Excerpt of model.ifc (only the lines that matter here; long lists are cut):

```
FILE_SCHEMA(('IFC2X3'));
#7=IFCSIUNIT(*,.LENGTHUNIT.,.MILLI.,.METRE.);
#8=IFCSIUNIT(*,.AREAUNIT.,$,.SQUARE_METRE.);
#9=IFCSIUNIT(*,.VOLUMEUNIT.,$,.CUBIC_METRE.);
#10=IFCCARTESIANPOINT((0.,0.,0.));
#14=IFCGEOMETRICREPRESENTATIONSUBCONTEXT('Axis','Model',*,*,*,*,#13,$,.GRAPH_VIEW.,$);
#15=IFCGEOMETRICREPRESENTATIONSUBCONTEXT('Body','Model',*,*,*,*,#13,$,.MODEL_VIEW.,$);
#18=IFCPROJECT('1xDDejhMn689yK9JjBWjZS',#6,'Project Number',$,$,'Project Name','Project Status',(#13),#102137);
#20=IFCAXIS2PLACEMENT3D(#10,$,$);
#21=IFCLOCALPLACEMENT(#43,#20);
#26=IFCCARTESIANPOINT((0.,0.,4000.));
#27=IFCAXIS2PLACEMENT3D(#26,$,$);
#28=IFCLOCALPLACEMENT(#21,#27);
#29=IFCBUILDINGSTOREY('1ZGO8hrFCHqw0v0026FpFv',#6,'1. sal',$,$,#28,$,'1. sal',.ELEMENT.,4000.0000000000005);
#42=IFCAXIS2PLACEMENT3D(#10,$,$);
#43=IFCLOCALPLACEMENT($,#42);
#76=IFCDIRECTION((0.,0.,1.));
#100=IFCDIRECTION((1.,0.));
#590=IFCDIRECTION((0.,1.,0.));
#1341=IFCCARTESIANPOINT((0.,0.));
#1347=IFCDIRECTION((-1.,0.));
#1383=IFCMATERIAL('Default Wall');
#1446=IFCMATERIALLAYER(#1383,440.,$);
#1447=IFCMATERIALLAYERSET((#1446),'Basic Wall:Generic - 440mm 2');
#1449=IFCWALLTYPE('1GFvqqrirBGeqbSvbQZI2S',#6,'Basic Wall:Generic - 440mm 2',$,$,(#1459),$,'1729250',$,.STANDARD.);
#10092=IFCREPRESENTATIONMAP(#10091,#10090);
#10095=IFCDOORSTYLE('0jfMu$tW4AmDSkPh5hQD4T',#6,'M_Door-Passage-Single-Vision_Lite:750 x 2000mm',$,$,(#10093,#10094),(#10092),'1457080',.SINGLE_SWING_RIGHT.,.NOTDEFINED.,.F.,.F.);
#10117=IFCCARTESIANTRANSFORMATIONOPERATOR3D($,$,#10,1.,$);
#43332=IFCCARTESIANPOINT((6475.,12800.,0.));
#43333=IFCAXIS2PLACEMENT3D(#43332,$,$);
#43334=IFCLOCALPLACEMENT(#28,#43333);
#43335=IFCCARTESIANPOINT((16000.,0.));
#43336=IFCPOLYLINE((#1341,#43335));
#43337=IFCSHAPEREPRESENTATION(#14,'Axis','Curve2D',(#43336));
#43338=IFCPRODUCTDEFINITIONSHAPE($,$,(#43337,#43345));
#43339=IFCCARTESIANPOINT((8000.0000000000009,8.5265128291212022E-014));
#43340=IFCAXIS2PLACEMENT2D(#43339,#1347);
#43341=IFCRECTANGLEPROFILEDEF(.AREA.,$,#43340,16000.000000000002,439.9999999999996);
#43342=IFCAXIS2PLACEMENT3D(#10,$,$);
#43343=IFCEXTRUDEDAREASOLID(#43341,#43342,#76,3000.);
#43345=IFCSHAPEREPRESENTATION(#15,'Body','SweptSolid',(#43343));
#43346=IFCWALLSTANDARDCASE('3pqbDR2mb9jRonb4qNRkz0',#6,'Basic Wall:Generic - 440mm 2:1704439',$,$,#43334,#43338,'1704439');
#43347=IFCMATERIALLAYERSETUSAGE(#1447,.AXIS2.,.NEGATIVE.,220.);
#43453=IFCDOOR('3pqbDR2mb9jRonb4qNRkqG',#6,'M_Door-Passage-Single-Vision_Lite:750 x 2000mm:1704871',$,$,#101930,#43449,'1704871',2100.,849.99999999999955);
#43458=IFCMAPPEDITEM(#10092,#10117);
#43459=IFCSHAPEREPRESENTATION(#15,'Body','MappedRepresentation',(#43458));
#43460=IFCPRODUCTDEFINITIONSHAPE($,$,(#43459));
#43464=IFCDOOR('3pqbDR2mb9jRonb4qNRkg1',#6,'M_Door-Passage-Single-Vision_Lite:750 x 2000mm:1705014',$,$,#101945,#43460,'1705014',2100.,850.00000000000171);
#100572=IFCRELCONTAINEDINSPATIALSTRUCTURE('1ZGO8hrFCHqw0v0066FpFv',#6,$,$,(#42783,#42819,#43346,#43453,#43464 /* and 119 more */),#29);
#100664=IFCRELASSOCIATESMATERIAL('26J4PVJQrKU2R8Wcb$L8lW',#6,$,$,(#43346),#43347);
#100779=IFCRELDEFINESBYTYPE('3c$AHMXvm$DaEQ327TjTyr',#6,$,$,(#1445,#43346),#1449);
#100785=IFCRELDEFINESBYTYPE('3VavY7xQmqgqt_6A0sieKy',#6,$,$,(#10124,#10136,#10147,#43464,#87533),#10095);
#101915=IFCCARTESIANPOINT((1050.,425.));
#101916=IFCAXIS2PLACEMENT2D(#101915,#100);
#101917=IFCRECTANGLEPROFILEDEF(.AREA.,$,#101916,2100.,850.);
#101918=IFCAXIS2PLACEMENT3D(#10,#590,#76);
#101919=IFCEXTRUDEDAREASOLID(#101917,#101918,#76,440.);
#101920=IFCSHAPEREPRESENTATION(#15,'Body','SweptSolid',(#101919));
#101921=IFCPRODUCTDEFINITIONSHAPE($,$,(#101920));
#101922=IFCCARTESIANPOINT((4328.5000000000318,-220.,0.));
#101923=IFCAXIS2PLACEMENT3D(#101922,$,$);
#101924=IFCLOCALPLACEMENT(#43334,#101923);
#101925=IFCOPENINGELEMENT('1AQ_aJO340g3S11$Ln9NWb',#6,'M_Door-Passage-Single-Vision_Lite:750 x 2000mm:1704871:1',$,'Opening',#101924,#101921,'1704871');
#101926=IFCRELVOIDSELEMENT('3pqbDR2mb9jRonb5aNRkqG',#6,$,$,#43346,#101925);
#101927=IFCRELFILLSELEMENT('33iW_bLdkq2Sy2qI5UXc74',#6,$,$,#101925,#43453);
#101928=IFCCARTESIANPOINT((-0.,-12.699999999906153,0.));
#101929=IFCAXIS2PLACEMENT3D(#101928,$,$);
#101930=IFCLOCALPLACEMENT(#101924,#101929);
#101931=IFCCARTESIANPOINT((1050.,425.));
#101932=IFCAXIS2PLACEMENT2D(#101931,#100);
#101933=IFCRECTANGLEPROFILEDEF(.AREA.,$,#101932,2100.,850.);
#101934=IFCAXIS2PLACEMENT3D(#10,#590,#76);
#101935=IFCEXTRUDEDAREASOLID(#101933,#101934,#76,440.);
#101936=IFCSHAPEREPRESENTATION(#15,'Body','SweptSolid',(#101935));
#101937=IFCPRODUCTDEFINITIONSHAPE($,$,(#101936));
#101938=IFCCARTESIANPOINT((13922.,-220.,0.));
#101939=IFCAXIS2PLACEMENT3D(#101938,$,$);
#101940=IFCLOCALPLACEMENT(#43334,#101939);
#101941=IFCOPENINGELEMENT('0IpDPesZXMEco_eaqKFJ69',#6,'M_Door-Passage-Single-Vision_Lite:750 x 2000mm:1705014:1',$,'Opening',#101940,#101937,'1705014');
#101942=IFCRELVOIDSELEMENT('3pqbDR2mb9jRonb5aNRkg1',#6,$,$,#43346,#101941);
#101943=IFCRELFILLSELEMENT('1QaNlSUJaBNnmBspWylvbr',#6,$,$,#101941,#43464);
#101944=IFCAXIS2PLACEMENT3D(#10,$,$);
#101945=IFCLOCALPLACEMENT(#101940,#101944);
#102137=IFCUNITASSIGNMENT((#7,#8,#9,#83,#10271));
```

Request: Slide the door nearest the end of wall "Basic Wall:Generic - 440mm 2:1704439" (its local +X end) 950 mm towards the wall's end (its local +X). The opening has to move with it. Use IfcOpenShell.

```python
import ifcopenshell
import ifcopenshell.api.geometry
import ifcopenshell.util.placement
import ifcopenshell.util.unit

model = ifcopenshell.open("model.ifc")
unit_scale = ifcopenshell.util.unit.calculate_unit_scale(model)

door = model.by_guid("3pqbDR2mb9jRonb4qNRkg1")
opening = door.FillsVoids[0].RelatingOpeningElement
wall = opening.VoidsElements[0].RelatingBuildingElement

wall_matrix = ifcopenshell.util.placement.get_local_placement(wall.ObjectPlacement)
shift = wall_matrix[:3, 0] * 0.95 / unit_scale
before = ifcopenshell.util.placement.get_local_placement(door.ObjectPlacement)[:3, 3].copy()

# The door is placed relative to its opening, so it follows when the opening moves.
matrix = ifcopenshell.util.placement.get_local_placement(opening.ObjectPlacement)
matrix[:3, 3] += shift
ifcopenshell.api.geometry.edit_object_placement(
    model, product=opening, matrix=matrix, is_si=False, should_transform_children=True
)

after = ifcopenshell.util.placement.get_local_placement(door.ObjectPlacement)[:3, 3]
print("door moved by", (after - before).round(3) + 0.0)

model.write("model_v2.ifc")
```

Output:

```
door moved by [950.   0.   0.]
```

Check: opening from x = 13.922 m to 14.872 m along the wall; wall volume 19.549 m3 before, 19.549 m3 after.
